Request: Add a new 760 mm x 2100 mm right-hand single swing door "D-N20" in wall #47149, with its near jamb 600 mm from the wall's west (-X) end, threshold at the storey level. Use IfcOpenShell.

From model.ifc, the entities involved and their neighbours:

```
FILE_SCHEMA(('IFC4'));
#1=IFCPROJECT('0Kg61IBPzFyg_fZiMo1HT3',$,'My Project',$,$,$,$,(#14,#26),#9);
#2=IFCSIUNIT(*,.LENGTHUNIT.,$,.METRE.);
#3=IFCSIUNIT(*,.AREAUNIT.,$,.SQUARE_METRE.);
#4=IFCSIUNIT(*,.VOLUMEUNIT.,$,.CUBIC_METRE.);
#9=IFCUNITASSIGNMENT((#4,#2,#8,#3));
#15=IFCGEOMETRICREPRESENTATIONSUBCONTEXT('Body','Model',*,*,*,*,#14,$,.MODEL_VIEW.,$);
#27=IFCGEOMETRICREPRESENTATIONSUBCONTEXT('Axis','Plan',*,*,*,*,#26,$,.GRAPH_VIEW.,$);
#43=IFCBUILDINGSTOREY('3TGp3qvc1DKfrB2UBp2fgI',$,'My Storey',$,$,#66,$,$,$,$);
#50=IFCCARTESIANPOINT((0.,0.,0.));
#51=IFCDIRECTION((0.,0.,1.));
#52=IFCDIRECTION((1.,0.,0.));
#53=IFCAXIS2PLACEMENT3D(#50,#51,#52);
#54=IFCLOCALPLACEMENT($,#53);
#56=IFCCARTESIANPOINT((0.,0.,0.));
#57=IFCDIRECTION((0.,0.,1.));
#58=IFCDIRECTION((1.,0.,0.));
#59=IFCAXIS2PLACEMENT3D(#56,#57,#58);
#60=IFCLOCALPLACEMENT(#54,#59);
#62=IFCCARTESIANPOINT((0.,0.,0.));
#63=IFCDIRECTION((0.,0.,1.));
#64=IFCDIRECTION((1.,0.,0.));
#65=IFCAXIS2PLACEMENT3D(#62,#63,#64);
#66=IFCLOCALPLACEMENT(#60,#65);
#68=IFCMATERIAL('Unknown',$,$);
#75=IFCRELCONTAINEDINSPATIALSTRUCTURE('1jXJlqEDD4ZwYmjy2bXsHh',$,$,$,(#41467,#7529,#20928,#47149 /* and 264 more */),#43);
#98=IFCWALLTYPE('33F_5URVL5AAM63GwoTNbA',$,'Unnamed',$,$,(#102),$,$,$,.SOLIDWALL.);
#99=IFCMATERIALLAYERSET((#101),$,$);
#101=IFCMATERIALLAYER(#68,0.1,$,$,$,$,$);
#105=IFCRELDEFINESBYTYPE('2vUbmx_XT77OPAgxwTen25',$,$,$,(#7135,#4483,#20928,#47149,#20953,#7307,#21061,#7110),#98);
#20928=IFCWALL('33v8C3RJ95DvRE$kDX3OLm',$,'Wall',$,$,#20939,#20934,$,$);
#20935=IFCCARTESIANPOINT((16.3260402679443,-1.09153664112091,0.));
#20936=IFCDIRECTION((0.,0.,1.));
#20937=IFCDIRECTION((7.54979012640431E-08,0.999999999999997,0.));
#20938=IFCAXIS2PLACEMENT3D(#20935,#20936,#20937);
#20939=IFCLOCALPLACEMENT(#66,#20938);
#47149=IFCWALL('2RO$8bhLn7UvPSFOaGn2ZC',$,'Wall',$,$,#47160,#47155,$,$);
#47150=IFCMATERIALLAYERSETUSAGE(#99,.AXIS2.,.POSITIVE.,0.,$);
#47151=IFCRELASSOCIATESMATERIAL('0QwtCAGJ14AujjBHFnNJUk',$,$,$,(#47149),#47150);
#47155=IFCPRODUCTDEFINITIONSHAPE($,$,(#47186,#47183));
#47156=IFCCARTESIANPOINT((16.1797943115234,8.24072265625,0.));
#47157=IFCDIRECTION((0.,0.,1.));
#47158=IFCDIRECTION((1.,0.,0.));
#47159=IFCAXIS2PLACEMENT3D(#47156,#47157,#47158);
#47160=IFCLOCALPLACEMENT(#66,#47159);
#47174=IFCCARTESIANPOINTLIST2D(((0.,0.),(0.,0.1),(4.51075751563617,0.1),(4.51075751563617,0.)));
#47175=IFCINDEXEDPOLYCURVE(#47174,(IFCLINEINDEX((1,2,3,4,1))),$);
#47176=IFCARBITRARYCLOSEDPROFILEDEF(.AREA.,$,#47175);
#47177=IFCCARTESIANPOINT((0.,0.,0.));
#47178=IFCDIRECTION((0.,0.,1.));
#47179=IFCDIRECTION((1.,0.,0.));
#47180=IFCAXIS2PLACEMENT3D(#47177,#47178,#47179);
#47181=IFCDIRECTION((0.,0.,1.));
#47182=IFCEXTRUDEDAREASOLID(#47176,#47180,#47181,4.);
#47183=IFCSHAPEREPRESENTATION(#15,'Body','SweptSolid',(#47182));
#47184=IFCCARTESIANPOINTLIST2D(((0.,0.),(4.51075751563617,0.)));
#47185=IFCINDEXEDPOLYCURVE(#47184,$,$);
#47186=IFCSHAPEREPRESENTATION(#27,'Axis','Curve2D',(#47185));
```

```python
import numpy as np
import ifcopenshell
import ifcopenshell.api.feature
import ifcopenshell.api.geometry
import ifcopenshell.api.root
import ifcopenshell.api.spatial
import ifcopenshell.geom
import ifcopenshell.util.element
import ifcopenshell.util.placement
import ifcopenshell.util.representation
import ifcopenshell.util.shape
import ifcopenshell.util.unit

model = ifcopenshell.open("model.ifc")
unit_scale = ifcopenshell.util.unit.calculate_unit_scale(model)
settings = ifcopenshell.geom.settings()


def volume(element):
    """Net volume in cubic metres, openings subtracted."""
    shape = ifcopenshell.geom.create_shape(settings, element)
    return ifcopenshell.util.shape.get_volume(shape.geometry)


wall = model.by_guid("2RO$8bhLn7UvPSFOaGn2ZC")
storey = ifcopenshell.util.element.get_container(wall, ifc_class="IfcBuildingStorey")
context = ifcopenshell.util.representation.get_context(model, "Model", "Body", "MODEL_VIEW")
before = volume(wall)

width, height, from_end, sill = 0.76, 2.1, 0.6, 0.0  # metres

# The wall runs along its own X axis, and the end named is its -X end.
wall_shape = ifcopenshell.geom.create_shape(settings, wall)
x, y, z = ifcopenshell.util.shape.get_vertices(wall_shape.geometry).T
start = x.min() + from_end
face, thickness = float(y.min()), float(y.max() - y.min())
wall_matrix = ifcopenshell.util.placement.get_local_placement(wall.ObjectPlacement)
level = ifcopenshell.util.placement.get_local_placement(storey.ObjectPlacement)[2, 3]


def in_wall(x, y):
    """Placement at x, y metres in the wall's axes, at sill height."""
    matrix = wall_matrix.copy()
    matrix[:, 3] = wall_matrix @ np.array([x / unit_scale, y / unit_scale, 0.0, 1.0])
    matrix[2, 3] = level + sill / unit_scale
    return matrix


# Opening: a box that overshoots both wall faces by 50 mm.
opening = ifcopenshell.api.root.create_entity(model, ifc_class="IfcOpeningElement", predefined_type="OPENING")
box = ifcopenshell.api.geometry.add_wall_representation(
    model, context=context, length=width, height=height, thickness=thickness + 0.1
)
ifcopenshell.api.geometry.assign_representation(model, product=opening, representation=box)
ifcopenshell.api.geometry.edit_object_placement(model, product=opening, matrix=in_wall(start, face - 0.05), is_si=False)
ifcopenshell.api.feature.add_feature(model, feature=opening, element=wall)

door = ifcopenshell.api.root.create_entity(model, ifc_class="IfcDoor", name="D-N20", predefined_type="DOOR")
door.OverallWidth, door.OverallHeight = width / unit_scale, height / unit_scale
door.OperationType = "SINGLE_SWING_RIGHT"
body = ifcopenshell.api.geometry.add_door_representation(
    model,
    context=context,
    overall_width=door.OverallWidth,
    overall_height=door.OverallHeight,
    operation_type="SINGLE_SWING_RIGHT",
    lining_properties={"LiningDepth": thickness / unit_scale, "ThresholdDepth": thickness / unit_scale},
)
ifcopenshell.api.geometry.assign_representation(model, product=door, representation=body)
ifcopenshell.api.spatial.assign_container(model, products=[door], relating_structure=storey)
ifcopenshell.api.feature.add_filling(model, opening=opening, element=door)

# The lining spans the wall, so the door starts at the wall face.
ifcopenshell.api.geometry.edit_object_placement(model, product=door, matrix=in_wall(start, face), is_si=False)

after = volume(wall)

print(f"wall volume {before:.3f} -> {after:.3f} m3")

model.write("model_rev.ifc")
```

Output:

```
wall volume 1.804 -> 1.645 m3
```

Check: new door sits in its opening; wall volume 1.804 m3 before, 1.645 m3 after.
